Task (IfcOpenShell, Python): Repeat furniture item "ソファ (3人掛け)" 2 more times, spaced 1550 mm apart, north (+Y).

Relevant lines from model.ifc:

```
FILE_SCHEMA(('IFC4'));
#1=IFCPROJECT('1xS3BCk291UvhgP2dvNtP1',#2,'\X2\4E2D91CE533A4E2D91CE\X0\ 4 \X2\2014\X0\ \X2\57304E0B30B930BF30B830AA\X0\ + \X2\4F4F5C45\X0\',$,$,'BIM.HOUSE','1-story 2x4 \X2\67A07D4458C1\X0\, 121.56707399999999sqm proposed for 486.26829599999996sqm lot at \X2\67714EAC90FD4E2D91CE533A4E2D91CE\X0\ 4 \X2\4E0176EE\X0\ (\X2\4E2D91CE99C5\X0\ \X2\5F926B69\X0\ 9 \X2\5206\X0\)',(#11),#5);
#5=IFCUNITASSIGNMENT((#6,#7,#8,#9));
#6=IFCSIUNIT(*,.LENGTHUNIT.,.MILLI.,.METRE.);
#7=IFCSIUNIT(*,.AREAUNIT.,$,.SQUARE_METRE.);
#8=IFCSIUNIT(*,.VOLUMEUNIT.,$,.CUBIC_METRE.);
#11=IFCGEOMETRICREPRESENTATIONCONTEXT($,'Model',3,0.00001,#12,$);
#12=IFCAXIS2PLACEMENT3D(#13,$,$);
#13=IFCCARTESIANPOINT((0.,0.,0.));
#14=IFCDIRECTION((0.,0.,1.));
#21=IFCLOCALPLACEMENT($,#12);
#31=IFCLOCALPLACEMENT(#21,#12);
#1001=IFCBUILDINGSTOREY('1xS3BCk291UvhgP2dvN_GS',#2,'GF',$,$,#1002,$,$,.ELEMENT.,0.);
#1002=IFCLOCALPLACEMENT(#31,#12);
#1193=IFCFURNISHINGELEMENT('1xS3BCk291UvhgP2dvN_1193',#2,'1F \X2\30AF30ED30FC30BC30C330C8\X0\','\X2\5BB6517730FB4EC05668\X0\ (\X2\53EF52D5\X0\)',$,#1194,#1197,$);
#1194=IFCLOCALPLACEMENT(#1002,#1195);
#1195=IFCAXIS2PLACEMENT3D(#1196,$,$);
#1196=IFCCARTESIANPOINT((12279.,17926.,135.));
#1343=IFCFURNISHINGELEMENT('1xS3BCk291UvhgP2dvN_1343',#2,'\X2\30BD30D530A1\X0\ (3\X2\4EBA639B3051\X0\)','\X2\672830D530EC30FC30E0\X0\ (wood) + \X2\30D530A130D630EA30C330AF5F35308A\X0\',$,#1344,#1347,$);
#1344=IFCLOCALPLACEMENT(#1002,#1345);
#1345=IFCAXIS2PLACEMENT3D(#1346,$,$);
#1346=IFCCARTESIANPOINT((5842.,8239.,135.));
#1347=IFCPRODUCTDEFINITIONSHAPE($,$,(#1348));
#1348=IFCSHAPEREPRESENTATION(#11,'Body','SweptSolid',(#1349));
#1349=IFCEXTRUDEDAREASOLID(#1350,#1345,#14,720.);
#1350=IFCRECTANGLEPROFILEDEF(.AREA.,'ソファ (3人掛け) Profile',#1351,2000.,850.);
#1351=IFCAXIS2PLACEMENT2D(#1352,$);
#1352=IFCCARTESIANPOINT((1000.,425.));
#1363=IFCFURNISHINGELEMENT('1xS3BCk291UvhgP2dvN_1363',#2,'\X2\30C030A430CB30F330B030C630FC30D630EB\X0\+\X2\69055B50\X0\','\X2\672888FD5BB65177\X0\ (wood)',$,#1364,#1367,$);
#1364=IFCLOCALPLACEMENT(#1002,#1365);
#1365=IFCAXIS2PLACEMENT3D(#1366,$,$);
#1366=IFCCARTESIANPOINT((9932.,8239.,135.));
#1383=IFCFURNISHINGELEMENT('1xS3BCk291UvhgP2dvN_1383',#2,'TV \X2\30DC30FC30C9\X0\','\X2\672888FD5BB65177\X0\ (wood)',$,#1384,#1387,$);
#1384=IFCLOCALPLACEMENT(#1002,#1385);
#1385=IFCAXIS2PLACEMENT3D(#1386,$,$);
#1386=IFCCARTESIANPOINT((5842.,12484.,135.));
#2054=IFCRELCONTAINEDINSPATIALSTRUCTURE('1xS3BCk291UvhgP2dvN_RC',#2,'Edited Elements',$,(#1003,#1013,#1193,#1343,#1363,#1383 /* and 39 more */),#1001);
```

```python
import numpy as np
import ifcopenshell
import ifcopenshell.api.geometry
import ifcopenshell.api.root
import ifcopenshell.util.element
import ifcopenshell.util.placement

model = ifcopenshell.open("model.ifc")


def reuse_history(source, copy):
    """copy_class also copies each property set's owner history, people and application; keep the originals."""
    for rel in copy.IsDefinedBy:
        if rel.is_a("IfcRelDefinesByProperties") and (history := rel.RelatingPropertyDefinition.OwnerHistory):
            rel.RelatingPropertyDefinition.OwnerHistory = source.OwnerHistory
            ifcopenshell.util.element.remove_deep2(model, history)


source = model.by_id(1343)
base = ifcopenshell.util.placement.get_local_placement(source.ObjectPlacement)
step = np.array([0.0, 1.0, 0.0]) * 1550.0

for i in range(1, 3):
    copy = ifcopenshell.api.root.copy_class(model, product=source)
    copy.Representation = ifcopenshell.util.element.copy_deep(
        model, source.Representation, exclude=["IfcGeometricRepresentationContext", "IfcRepresentationMap"]
    )
    reuse_history(source, copy)
    matrix = base.copy()
    matrix[:3, 3] += i * step
    print("added at", matrix[:3, 3].round(3) + 0.0)
    ifcopenshell.api.geometry.edit_object_placement(model, product=copy, matrix=matrix, is_si=False)

model.write("model_edited.ifc")
```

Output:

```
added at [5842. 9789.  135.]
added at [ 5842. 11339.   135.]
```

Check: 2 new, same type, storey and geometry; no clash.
